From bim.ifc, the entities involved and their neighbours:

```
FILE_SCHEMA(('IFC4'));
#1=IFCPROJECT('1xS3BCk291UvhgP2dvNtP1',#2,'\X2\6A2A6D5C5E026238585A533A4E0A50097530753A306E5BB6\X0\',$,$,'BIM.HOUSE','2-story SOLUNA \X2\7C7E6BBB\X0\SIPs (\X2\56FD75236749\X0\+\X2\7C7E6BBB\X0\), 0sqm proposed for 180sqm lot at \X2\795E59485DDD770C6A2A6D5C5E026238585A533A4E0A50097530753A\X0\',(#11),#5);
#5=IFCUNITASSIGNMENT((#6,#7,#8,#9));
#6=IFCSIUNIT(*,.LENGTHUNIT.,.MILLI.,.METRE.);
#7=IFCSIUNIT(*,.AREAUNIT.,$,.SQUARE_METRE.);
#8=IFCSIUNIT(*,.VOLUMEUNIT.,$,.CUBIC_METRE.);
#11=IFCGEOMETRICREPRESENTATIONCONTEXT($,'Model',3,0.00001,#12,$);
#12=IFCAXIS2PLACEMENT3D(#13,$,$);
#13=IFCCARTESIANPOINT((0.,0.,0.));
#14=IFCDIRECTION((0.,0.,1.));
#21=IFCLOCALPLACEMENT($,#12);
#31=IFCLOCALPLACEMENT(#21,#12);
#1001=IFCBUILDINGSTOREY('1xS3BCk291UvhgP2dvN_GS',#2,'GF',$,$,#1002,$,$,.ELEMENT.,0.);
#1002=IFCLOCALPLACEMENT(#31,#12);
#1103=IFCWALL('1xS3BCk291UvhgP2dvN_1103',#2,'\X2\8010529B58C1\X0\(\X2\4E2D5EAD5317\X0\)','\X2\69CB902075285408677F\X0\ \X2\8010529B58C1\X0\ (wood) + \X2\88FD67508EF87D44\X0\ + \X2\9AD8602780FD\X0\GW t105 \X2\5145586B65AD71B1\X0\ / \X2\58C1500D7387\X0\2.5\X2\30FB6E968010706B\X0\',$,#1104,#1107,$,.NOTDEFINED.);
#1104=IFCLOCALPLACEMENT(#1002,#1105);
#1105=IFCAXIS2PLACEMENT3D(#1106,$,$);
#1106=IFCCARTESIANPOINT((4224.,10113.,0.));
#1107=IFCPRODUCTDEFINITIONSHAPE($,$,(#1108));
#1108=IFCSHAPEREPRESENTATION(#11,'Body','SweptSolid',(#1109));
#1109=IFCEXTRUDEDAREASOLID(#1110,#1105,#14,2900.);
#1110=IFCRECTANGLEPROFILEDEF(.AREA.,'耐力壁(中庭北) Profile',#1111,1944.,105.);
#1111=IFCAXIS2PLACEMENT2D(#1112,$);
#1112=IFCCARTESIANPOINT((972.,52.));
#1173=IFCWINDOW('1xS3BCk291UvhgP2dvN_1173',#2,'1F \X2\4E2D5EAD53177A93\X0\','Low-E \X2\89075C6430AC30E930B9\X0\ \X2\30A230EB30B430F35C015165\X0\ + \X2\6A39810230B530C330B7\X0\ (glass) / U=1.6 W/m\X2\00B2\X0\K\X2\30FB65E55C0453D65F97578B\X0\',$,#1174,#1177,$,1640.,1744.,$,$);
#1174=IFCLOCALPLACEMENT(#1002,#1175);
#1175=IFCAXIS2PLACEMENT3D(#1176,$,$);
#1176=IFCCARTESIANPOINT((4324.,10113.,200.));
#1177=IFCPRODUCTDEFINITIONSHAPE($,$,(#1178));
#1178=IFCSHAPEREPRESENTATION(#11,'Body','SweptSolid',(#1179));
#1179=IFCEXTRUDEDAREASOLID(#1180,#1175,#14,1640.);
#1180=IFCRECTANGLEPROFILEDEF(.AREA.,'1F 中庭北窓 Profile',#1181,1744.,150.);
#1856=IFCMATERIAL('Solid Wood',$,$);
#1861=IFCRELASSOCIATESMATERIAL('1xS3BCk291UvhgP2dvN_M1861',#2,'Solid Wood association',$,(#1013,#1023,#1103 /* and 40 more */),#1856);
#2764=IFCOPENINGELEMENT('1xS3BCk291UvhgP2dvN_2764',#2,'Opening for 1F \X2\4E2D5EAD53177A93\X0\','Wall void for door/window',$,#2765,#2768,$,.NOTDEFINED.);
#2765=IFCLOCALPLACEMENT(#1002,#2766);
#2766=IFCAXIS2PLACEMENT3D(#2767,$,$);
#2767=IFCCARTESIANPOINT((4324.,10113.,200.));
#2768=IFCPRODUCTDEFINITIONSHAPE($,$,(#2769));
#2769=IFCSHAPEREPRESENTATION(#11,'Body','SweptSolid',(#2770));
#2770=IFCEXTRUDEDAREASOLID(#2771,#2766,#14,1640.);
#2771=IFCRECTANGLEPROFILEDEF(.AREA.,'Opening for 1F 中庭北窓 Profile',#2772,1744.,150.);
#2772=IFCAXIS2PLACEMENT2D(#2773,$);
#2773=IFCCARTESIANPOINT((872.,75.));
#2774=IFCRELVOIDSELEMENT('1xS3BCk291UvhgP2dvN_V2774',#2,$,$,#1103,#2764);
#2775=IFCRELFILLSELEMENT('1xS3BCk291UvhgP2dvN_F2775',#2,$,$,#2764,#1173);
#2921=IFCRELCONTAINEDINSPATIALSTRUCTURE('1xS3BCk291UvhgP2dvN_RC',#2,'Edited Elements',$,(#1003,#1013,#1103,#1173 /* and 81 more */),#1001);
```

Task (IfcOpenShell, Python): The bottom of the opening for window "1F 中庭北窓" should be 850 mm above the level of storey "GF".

```python
import numpy as np
import ifcopenshell
import ifcopenshell.api.geometry
import ifcopenshell.geom
import ifcopenshell.util.element
import ifcopenshell.util.placement
import ifcopenshell.util.shape
import ifcopenshell.util.unit

model = ifcopenshell.open("bim.ifc")
unit_scale = ifcopenshell.util.unit.calculate_unit_scale(model)

window = model.by_id(1173)
opening = window.FillsVoids[0].RelatingOpeningElement
storey = ifcopenshell.util.element.get_container(window, ifc_class="IfcBuildingStorey")
level = ifcopenshell.util.placement.get_local_placement(storey.ObjectPlacement)[2, 3]

# The opening's origin need not be at the sill, so measure its lowest point.
shape = ifcopenshell.geom.create_shape(ifcopenshell.geom.settings(), opening)
bottom = ifcopenshell.util.shape.get_shape_bottom_elevation(shape, shape.geometry) / unit_scale
dz = level + 850.0 - bottom

shift = np.array([0.0, 0.0, dz])
# The window is not placed relative to its opening, so move both.
for product in (opening, window):
    matrix = ifcopenshell.util.placement.get_local_placement(product.ObjectPlacement)
    matrix[:3, 3] += shift
    ifcopenshell.api.geometry.edit_object_placement(model, product=product, matrix=matrix, is_si=False)

print(f"moved by {dz * unit_scale:+.3f} m")

model.write("bim_edited.ifc")
```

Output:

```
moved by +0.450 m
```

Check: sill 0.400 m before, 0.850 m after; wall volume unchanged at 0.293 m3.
